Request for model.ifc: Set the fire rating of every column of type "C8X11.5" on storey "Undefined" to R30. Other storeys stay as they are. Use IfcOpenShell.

First a look at what the model holds.

```python
import ifcopenshell
import ifcopenshell.util.element

model = ifcopenshell.open("model.ifc")
print(model.schema)
storey = next(s for s in model.by_type("IfcBuildingStorey") if s.Name == "Undefined")
columns = [e for e in ifcopenshell.util.element.get_decomposition(storey) if e.is_a("IfcColumn")]
seen = {}
for e in columns:
    element_type = ifcopenshell.util.element.get_type(e)
    key = (element_type.Name if element_type != e and element_type else None, ifcopenshell.util.element.get_pset(e, "Pset_ColumnCommon", "FireRating"))
    seen[key] = seen.get(key, 0) + 1
for (name, value), count in sorted(seen.items(), key=str):
    print(count, "x", name, "|", value)
```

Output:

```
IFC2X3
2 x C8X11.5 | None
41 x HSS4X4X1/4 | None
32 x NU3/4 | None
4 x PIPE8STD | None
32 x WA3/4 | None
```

```python
import ifcopenshell
import ifcopenshell.api.pset
import ifcopenshell.util.element

model = ifcopenshell.open("model.ifc")

storey = next(s for s in model.by_type("IfcBuildingStorey") if s.Name == "Undefined")
columns = [e for e in ifcopenshell.util.element.get_decomposition(storey) if e.is_a("IfcColumn")]

count = 0
for e in columns:
    element_type = ifcopenshell.util.element.get_type(e)
    if element_type in (None, e) or element_type.Name != "C8X11.5":
        continue
    # add_pset returns the element's existing set when there is one.
    pset = ifcopenshell.api.pset.add_pset(model, product=e, name="Pset_ColumnCommon")
    ifcopenshell.api.pset.edit_pset(model, pset=pset, properties={"FireRating": "R30"})
    count += 1

print(count, "columns updated")

model.write("model_updated.ifc")
```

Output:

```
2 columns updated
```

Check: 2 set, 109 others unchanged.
